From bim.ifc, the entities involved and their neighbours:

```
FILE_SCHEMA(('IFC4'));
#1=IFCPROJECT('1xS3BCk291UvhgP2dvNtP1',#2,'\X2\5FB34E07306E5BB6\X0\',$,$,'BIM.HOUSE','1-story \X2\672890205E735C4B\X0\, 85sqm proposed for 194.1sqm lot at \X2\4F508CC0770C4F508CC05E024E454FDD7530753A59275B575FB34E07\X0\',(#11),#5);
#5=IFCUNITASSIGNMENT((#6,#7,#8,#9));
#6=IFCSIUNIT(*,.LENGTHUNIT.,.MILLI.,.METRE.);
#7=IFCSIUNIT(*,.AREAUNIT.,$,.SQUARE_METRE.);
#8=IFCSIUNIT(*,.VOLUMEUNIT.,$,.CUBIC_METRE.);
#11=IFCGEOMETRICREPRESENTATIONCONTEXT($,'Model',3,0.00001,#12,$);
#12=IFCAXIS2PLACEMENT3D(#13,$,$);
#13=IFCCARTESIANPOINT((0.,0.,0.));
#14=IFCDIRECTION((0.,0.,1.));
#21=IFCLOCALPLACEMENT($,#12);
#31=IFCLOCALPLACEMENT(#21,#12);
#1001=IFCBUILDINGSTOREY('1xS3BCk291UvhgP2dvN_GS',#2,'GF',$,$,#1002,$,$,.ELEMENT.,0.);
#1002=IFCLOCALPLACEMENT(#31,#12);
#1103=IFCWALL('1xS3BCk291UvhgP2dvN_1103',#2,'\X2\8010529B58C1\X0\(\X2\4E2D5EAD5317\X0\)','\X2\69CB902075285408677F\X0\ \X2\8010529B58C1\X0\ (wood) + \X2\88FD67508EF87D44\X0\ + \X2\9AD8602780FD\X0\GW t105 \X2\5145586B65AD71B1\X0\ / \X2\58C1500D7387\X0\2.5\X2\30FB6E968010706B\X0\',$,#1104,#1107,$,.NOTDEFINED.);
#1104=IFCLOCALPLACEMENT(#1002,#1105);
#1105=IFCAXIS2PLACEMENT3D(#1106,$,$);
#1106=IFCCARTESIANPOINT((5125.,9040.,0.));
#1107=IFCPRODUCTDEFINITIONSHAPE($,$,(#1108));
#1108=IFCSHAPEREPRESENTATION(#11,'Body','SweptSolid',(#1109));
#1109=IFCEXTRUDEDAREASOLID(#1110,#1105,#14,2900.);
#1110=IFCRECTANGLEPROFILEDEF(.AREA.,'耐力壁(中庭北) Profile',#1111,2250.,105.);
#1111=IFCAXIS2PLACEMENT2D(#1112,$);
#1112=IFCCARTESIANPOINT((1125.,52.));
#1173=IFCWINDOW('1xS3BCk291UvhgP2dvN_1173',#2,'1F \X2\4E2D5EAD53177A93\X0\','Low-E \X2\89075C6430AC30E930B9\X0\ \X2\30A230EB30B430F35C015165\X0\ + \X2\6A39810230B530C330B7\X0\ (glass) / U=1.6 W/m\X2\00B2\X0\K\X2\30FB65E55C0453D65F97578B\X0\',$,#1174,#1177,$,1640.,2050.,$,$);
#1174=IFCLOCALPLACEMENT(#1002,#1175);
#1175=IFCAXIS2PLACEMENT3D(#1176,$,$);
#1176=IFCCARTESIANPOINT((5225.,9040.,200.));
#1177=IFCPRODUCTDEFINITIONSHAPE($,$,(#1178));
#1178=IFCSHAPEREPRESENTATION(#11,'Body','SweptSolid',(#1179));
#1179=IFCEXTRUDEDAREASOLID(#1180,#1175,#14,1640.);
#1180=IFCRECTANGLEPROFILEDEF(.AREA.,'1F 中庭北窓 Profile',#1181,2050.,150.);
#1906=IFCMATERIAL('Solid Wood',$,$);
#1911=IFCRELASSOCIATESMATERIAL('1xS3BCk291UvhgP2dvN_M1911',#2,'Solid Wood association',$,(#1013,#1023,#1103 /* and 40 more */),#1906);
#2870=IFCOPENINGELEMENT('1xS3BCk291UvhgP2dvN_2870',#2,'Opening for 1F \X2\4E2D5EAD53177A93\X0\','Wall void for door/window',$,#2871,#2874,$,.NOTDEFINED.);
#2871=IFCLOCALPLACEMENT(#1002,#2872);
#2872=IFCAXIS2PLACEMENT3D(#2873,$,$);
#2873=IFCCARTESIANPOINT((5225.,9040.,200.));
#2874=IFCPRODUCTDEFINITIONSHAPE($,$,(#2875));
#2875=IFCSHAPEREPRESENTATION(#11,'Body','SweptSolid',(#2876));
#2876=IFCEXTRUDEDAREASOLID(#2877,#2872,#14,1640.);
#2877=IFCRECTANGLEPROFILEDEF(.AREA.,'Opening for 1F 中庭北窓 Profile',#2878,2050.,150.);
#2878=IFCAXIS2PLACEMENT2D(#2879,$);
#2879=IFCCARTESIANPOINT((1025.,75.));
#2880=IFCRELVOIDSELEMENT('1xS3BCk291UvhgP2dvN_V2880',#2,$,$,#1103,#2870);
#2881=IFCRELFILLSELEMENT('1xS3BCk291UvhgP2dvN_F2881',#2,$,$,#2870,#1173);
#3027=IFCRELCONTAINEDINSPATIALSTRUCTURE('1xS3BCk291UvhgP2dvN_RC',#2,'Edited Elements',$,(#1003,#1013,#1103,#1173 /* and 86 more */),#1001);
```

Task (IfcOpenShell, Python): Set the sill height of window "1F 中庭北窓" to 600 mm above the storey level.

```python
import numpy as np
import ifcopenshell
import ifcopenshell.api.geometry
import ifcopenshell.geom
import ifcopenshell.util.element
import ifcopenshell.util.placement
import ifcopenshell.util.shape
import ifcopenshell.util.unit

model = ifcopenshell.open("bim.ifc")
unit_scale = ifcopenshell.util.unit.calculate_unit_scale(model)

window = model.by_guid("1xS3BCk291UvhgP2dvN_1173")
opening = window.FillsVoids[0].RelatingOpeningElement
storey = ifcopenshell.util.element.get_container(window, ifc_class="IfcBuildingStorey")
level = ifcopenshell.util.placement.get_local_placement(storey.ObjectPlacement)[2, 3]

# The opening's origin need not be at the sill, so measure its lowest point.
shape = ifcopenshell.geom.create_shape(ifcopenshell.geom.settings(), opening)
bottom = ifcopenshell.util.shape.get_shape_bottom_elevation(shape, shape.geometry) / unit_scale
dz = level + 600.0 - bottom

shift = np.array([0.0, 0.0, dz])
# The window is not placed relative to its opening, so move both.
for product in (opening, window):
    matrix = ifcopenshell.util.placement.get_local_placement(product.ObjectPlacement)
    matrix[:3, 3] += shift
    ifcopenshell.api.geometry.edit_object_placement(model, product=product, matrix=matrix, is_si=False)

print(f"moved by {dz * unit_scale:+.3f} m")

model.write("bim_rev.ifc")
```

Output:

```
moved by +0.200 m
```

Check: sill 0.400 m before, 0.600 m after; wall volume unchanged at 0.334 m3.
